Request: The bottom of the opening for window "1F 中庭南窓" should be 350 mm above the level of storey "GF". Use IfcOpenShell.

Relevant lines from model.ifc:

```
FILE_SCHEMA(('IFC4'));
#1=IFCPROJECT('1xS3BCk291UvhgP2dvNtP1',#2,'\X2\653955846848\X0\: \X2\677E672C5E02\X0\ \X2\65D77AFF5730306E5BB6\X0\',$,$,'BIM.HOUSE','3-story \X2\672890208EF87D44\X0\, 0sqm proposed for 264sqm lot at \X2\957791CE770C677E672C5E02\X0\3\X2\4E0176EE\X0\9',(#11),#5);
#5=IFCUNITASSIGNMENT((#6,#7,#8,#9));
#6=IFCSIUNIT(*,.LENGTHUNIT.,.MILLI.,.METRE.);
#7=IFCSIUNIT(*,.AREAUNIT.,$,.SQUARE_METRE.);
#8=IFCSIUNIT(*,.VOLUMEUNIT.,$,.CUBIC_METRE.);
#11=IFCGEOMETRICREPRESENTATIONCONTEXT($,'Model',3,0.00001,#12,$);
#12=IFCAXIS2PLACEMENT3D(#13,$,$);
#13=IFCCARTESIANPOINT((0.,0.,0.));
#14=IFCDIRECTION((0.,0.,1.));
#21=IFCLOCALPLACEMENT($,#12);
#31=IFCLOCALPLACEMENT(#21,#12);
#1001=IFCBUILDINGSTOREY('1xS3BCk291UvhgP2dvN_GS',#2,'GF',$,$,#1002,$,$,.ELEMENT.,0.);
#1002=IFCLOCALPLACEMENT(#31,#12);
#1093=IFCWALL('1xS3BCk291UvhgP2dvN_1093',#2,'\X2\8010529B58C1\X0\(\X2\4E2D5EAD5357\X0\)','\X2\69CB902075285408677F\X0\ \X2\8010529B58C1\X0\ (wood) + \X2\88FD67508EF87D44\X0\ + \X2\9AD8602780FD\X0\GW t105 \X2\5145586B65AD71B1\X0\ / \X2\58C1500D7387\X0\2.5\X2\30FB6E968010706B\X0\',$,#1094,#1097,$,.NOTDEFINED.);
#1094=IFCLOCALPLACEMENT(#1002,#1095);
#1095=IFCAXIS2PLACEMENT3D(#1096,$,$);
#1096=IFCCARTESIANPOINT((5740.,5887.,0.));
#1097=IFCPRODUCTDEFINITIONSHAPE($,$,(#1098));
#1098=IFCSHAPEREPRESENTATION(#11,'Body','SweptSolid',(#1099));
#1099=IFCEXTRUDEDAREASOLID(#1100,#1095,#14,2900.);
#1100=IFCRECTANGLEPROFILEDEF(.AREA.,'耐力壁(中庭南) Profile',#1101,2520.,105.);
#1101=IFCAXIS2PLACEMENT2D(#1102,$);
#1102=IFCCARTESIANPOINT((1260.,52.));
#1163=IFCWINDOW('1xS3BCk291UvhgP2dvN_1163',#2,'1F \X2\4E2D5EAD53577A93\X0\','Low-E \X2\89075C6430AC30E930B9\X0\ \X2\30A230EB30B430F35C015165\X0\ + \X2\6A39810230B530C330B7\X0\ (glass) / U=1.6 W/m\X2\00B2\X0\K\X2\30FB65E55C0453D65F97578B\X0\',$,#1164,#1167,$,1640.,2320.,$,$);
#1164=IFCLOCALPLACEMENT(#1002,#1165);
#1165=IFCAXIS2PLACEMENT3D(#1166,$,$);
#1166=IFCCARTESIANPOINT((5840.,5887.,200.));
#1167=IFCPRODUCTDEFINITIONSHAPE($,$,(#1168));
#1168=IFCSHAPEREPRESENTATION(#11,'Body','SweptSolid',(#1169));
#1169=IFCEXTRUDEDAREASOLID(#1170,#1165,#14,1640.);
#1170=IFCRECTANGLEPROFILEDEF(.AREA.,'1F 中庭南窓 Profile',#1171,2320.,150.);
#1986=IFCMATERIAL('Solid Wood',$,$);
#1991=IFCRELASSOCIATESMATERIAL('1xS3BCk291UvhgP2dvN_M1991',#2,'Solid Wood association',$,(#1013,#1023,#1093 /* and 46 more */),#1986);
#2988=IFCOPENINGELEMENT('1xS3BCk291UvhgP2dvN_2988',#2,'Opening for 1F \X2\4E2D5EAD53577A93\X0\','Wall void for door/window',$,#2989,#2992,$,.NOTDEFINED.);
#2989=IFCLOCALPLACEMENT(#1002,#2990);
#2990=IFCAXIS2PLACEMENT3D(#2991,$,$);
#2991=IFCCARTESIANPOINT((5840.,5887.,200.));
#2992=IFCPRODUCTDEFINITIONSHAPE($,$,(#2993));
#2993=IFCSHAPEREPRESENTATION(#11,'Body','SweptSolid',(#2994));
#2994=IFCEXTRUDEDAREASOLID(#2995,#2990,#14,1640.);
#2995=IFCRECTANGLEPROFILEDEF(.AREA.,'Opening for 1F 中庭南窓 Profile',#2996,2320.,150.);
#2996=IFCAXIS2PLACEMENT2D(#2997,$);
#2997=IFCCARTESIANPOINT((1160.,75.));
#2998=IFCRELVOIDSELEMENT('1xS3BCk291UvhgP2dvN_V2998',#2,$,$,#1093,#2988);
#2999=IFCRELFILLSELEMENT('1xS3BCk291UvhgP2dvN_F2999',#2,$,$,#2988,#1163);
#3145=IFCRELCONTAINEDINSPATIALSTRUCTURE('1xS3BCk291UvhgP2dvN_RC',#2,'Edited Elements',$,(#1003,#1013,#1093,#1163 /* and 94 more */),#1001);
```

```python
import numpy as np
import ifcopenshell
import ifcopenshell.api.geometry
import ifcopenshell.geom
import ifcopenshell.util.element
import ifcopenshell.util.placement
import ifcopenshell.util.shape
import ifcopenshell.util.unit

model = ifcopenshell.open("model.ifc")
unit_scale = ifcopenshell.util.unit.calculate_unit_scale(model)

window = model.by_guid("1xS3BCk291UvhgP2dvN_1163")
opening = window.FillsVoids[0].RelatingOpeningElement
storey = ifcopenshell.util.element.get_container(window, ifc_class="IfcBuildingStorey")
level = ifcopenshell.util.placement.get_local_placement(storey.ObjectPlacement)[2, 3]

# The opening's origin need not be at the sill, so measure its lowest point.
shape = ifcopenshell.geom.create_shape(ifcopenshell.geom.settings(), opening)
bottom = ifcopenshell.util.shape.get_shape_bottom_elevation(shape, shape.geometry) / unit_scale
dz = level + 0.35 / unit_scale - bottom

shift = np.array([0.0, 0.0, dz])
# The window is not placed relative to its opening, so move both.
for product in (opening, window):
    matrix = ifcopenshell.util.placement.get_local_placement(product.ObjectPlacement)
    matrix[:3, 3] += shift
    ifcopenshell.api.geometry.edit_object_placement(model, product=product, matrix=matrix, is_si=False)

print(f"moved by {dz * unit_scale:+.3f} m")

model.write("model_updated.ifc")
```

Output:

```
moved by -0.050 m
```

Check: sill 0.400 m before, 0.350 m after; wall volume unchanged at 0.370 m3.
